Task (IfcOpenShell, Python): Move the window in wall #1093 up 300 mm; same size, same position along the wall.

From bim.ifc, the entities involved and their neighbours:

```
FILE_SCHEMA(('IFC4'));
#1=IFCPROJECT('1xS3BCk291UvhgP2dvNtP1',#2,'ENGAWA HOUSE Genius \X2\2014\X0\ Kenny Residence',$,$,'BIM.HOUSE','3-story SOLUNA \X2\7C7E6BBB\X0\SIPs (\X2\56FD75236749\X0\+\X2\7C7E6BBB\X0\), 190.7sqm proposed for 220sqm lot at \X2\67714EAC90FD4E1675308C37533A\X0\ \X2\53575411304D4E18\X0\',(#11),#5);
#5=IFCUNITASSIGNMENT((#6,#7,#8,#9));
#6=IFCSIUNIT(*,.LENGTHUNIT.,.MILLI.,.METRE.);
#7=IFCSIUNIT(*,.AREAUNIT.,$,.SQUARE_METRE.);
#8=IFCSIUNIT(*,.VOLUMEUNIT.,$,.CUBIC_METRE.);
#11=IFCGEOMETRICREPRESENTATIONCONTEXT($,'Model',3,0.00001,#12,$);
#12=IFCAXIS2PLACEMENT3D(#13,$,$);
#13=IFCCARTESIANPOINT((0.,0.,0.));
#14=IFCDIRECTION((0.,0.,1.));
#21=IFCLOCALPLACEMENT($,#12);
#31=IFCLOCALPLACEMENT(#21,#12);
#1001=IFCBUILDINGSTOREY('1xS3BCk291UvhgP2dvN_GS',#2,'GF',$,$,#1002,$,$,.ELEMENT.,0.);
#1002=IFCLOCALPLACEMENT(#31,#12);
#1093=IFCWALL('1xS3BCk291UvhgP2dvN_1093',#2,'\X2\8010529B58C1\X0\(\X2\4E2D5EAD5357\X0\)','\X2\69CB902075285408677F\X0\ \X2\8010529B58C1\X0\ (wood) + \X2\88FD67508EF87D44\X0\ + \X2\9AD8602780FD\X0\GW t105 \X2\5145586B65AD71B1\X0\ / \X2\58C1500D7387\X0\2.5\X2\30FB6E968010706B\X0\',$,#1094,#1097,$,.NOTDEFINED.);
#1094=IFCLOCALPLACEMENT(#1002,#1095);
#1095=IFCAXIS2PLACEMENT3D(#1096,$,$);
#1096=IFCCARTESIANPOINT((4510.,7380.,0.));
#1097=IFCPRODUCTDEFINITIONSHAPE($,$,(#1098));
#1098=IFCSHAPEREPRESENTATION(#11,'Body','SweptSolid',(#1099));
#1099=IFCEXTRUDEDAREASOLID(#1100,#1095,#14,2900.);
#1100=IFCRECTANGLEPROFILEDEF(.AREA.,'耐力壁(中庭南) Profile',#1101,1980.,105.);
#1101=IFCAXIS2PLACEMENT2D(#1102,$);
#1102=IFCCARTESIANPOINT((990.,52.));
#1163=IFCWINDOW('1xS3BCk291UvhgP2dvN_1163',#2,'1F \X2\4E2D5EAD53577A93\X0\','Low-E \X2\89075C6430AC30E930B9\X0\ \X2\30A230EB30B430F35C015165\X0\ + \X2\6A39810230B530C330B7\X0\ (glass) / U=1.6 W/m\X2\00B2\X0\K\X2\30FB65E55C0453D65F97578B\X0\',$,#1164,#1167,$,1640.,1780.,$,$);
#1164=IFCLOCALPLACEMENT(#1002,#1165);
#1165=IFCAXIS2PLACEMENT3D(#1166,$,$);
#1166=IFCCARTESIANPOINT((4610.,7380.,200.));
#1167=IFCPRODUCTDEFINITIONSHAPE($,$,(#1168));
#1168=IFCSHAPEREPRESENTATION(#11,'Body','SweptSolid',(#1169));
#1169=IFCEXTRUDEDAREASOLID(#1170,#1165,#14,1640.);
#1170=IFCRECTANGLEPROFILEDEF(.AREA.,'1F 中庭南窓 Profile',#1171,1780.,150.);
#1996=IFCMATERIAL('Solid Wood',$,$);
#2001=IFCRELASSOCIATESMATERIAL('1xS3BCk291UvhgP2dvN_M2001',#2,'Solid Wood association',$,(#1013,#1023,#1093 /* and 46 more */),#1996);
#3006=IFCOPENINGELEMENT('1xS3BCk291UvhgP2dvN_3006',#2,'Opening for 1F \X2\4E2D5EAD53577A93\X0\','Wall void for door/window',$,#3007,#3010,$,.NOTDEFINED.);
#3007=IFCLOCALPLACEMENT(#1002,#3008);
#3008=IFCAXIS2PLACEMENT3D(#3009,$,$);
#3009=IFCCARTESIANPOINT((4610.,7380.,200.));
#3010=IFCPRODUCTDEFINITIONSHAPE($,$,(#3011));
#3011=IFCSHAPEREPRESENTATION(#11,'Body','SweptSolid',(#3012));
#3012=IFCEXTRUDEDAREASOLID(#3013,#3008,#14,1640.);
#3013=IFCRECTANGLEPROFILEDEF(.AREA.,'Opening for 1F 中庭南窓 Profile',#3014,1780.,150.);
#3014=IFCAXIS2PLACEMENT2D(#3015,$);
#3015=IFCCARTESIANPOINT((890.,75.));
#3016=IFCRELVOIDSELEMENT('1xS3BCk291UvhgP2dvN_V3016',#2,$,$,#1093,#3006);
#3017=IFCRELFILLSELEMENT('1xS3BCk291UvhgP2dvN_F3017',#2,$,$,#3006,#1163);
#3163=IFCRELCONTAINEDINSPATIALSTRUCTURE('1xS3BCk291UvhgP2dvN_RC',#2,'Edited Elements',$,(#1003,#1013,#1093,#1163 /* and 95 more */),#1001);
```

```python
import numpy as np
import ifcopenshell
import ifcopenshell.api.geometry
import ifcopenshell.util.placement
import ifcopenshell.util.unit

model = ifcopenshell.open("bim.ifc")
unit_scale = ifcopenshell.util.unit.calculate_unit_scale(model)

window = model.by_guid("1xS3BCk291UvhgP2dvN_1163")
opening = window.FillsVoids[0].RelatingOpeningElement
dz = 0.3 / unit_scale

shift = np.array([0.0, 0.0, dz])
# The window is not placed relative to its opening, so move both.
for product in (opening, window):
    matrix = ifcopenshell.util.placement.get_local_placement(product.ObjectPlacement)
    matrix[:3, 3] += shift
    ifcopenshell.api.geometry.edit_object_placement(model, product=product, matrix=matrix, is_si=False)

print(f"moved by {dz * unit_scale:+.3f} m")

model.write("bim_v2.ifc")
```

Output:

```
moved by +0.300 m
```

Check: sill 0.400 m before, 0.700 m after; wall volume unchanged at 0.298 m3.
